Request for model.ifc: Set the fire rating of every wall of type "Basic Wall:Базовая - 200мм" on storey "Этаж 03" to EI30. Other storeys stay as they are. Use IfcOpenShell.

First a look at what the model holds.

```python
import ifcopenshell
import ifcopenshell.util.element

model = ifcopenshell.open("model.ifc")
print(model.schema)
storey = next(s for s in model.by_type("IfcBuildingStorey") if s.Name == "Этаж 03")
walls = [e for e in ifcopenshell.util.element.get_decomposition(storey) if e.is_a("IfcWall")]
seen = {}
for e in walls:
    element_type = ifcopenshell.util.element.get_type(e)
    key = (element_type.Name if element_type != e and element_type else None, ifcopenshell.util.element.get_pset(e, "Pset_WallCommon", "FireRating"))
    seen[key] = seen.get(key, 0) + 1
for (name, value), count in sorted(seen.items(), key=str):
    print(count, "x", name, "|", value)
```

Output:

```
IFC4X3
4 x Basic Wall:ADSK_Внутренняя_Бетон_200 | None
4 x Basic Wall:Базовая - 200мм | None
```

```python
import ifcopenshell
import ifcopenshell.api.pset
import ifcopenshell.util.element

model = ifcopenshell.open("model.ifc")

storey = next(s for s in model.by_type("IfcBuildingStorey") if s.Name == "Этаж 03")
walls = [e for e in ifcopenshell.util.element.get_decomposition(storey) if e.is_a("IfcWall")]

count = 0
for e in walls:
    element_type = ifcopenshell.util.element.get_type(e)
    if element_type in (None, e) or element_type.Name != "Basic Wall:Базовая - 200мм":
        continue
    # add_pset returns the element's existing set when there is one.
    pset = ifcopenshell.api.pset.add_pset(model, product=e, name="Pset_WallCommon")
    ifcopenshell.api.pset.edit_pset(model, pset=pset, properties={"FireRating": "EI30"})
    count += 1

print(count, "walls updated")

model.write("model_rev.ifc")
```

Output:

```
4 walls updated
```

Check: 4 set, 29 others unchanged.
